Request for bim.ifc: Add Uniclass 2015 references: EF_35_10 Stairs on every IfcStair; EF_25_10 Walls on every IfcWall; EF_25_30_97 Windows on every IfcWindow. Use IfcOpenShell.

First a look at what the model holds.

```python
import ifcopenshell

model = ifcopenshell.open("bim.ifc")
print(model.schema)
print("classifications:", [c.Name for c in model.by_type("IfcClassification")])
for ifc_class in ("IfcDoor", "IfcRoof", "IfcStair", "IfcWall", "IfcWindow"):
    print(ifc_class, len(model.by_type(ifc_class)))
```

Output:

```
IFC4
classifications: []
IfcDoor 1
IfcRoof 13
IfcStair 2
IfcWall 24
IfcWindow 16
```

```python
import ifcopenshell
import ifcopenshell.api.classification

model = ifcopenshell.open("bim.ifc")

system = ifcopenshell.api.classification.add_classification(model, classification="Uniclass 2015")

codes = {
    "IfcStair": ("EF_35_10", "Stairs"),
    "IfcWall": ("EF_25_10", "Walls"),
    "IfcWindow": ("EF_25_30_97", "Windows"),
}
for ifc_class, (code, name) in codes.items():
    products = model.by_type(ifc_class)
    ifcopenshell.api.classification.add_reference(
        model, products=products, classification=system, identification=code, name=name
    )
    print(code, len(products))

model.write("bim_updated.ifc")
```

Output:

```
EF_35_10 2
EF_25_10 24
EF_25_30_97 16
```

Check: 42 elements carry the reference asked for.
